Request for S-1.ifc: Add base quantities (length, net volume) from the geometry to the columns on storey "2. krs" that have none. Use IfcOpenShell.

First a look at what the model holds.

```python
import ifcopenshell
import ifcopenshell.util.element
import ifcopenshell.util.unit

model = ifcopenshell.open("S-1.ifc")
print(model.schema)
for unit_type in ("LENGTHUNIT", "AREAUNIT", "VOLUMEUNIT"):
    print(unit_type, ifcopenshell.util.unit.calculate_unit_scale(model, unit_type))
storey = next(s for s in model.by_type("IfcBuildingStorey") if s.Name == "2. krs")
columns = [e for e in ifcopenshell.util.element.get_decomposition(storey) if e.is_a("IfcColumn")]
for e in sorted(columns, key=lambda e: e.id()):
    print(e.id(), e.is_a(), e.Name, list(ifcopenshell.util.element.get_psets(e, qtos_only=True)), sep=" | ")
```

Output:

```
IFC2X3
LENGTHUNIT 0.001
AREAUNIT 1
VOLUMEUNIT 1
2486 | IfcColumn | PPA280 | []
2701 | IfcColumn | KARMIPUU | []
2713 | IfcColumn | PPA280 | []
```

```python
import ifcopenshell
import ifcopenshell.api.pset
import ifcopenshell.geom
import ifcopenshell.util.element
import ifcopenshell.util.shape
import ifcopenshell.util.unit

model = ifcopenshell.open("S-1.ifc")
unit_scale = ifcopenshell.util.unit.calculate_unit_scale(model)
volume_scale = ifcopenshell.util.unit.calculate_unit_scale(model, "VOLUMEUNIT")
settings = ifcopenshell.geom.settings()

storey = next(s for s in model.by_type("IfcBuildingStorey") if s.Name == "2. krs")
columns = [e for e in ifcopenshell.util.element.get_decomposition(storey) if e.is_a("IfcColumn")]

for e in sorted(columns, key=lambda e: e.id()):
    if ifcopenshell.util.element.get_psets(e, qtos_only=True, should_inherit=False):
        continue
    # Geometry comes back in metres, in the element's own axes.
    shape = ifcopenshell.geom.create_shape(settings, e)
    values = {
        "Length": ifcopenshell.util.shape.get_z(shape.geometry) / unit_scale,
        "NetVolume": ifcopenshell.util.shape.get_volume(shape.geometry) / volume_scale,
    }
    qto = ifcopenshell.api.pset.add_qto(model, product=e, name="BaseQuantities")
    ifcopenshell.api.pset.edit_qto(model, qto=qto, properties=values)
    print(e.id(), {k: round(v, 3) for k, v in values.items()})

model.write("S-1-out.ifc")
```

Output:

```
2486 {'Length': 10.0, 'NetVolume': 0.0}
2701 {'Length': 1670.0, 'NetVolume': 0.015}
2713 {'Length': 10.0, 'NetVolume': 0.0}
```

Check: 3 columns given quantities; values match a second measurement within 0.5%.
